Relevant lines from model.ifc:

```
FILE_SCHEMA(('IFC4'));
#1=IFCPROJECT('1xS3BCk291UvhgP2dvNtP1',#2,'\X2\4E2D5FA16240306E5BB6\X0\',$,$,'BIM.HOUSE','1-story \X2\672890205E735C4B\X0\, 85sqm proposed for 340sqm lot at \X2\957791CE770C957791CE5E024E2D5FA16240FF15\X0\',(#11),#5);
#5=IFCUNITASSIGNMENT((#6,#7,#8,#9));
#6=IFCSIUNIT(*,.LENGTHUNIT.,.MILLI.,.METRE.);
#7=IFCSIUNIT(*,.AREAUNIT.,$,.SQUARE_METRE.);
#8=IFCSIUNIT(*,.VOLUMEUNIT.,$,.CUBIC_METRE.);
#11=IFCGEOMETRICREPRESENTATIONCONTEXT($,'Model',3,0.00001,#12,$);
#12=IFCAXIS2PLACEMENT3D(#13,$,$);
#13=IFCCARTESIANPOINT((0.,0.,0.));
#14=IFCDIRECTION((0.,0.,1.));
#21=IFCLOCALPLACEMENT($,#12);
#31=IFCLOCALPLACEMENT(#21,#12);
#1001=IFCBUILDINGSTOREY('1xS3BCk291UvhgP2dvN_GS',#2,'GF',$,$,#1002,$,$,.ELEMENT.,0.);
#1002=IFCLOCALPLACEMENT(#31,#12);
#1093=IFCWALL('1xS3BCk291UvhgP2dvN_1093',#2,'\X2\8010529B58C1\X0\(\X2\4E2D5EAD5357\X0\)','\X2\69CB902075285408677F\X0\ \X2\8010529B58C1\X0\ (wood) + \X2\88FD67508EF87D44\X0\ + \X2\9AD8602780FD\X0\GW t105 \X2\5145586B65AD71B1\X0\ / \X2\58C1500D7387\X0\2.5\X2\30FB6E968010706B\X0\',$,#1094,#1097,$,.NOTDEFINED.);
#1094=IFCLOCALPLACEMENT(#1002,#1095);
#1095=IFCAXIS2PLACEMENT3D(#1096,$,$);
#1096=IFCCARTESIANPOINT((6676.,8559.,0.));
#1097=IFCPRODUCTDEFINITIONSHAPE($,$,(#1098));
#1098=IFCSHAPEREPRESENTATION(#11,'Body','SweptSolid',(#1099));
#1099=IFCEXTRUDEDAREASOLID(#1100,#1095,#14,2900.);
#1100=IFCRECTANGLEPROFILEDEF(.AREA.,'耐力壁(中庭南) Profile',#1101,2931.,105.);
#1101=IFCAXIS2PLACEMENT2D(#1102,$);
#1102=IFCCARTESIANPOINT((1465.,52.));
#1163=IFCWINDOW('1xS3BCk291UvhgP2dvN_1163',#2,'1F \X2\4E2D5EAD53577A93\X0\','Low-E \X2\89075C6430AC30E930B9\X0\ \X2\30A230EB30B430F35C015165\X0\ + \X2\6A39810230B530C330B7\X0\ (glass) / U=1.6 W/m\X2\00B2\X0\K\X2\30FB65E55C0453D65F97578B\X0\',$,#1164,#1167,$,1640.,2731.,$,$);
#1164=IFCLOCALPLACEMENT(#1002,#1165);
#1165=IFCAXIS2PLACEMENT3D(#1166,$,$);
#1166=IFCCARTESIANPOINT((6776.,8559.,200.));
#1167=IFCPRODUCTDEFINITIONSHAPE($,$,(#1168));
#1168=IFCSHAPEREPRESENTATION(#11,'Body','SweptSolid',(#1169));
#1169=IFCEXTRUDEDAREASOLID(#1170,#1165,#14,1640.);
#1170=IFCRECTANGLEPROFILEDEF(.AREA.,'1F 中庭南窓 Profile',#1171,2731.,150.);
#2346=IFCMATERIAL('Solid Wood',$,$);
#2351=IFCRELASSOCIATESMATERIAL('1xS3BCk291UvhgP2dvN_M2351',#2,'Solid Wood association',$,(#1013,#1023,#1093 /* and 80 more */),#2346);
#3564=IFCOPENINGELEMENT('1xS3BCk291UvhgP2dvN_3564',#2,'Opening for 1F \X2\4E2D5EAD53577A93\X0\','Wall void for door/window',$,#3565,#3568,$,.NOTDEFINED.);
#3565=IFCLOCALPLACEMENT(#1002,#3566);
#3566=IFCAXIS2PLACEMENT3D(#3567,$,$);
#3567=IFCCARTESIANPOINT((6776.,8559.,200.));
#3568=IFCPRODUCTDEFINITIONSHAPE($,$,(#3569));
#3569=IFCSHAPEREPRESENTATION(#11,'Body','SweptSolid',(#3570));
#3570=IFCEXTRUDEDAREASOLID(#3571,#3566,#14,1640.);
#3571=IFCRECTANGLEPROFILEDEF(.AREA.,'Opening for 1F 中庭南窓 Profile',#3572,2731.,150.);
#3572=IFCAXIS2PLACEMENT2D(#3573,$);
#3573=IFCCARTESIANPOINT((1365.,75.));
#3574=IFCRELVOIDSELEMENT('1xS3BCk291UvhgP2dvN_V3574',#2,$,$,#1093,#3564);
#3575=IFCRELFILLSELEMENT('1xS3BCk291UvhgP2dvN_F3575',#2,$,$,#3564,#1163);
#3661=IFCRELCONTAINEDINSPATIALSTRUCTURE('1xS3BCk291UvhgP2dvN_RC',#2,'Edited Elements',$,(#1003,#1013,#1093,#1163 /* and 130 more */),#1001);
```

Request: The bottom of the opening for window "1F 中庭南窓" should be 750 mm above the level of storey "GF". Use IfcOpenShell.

```python
import numpy as np
import ifcopenshell
import ifcopenshell.api.geometry
import ifcopenshell.geom
import ifcopenshell.util.element
import ifcopenshell.util.placement
import ifcopenshell.util.shape
import ifcopenshell.util.unit

model = ifcopenshell.open("model.ifc")
unit_scale = ifcopenshell.util.unit.calculate_unit_scale(model)

window = model.by_guid("1xS3BCk291UvhgP2dvN_1163")
opening = window.FillsVoids[0].RelatingOpeningElement
storey = ifcopenshell.util.element.get_container(window, ifc_class="IfcBuildingStorey")
level = ifcopenshell.util.placement.get_local_placement(storey.ObjectPlacement)[2, 3]

# The opening's origin need not be at the sill, so measure its lowest point.
shape = ifcopenshell.geom.create_shape(ifcopenshell.geom.settings(), opening)
bottom = ifcopenshell.util.shape.get_shape_bottom_elevation(shape, shape.geometry) / unit_scale
dz = level + 0.75 / unit_scale - bottom

shift = np.array([0.0, 0.0, dz])
# The window is not placed relative to its opening, so move both.
for product in (opening, window):
    matrix = ifcopenshell.util.placement.get_local_placement(product.ObjectPlacement)
    matrix[:3, 3] += shift
    ifcopenshell.api.geometry.edit_object_placement(model, product=product, matrix=matrix, is_si=False)

print(f"moved by {dz * unit_scale:+.3f} m")

model.write("model-out.ifc")
```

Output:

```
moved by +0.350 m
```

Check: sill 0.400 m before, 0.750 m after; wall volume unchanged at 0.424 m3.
